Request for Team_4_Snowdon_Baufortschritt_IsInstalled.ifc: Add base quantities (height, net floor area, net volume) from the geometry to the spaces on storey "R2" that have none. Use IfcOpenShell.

First a look at what the model holds.

```python
import ifcopenshell
import ifcopenshell.util.element
import ifcopenshell.util.unit

model = ifcopenshell.open("Team_4_Snowdon_Baufortschritt_IsInstalled.ifc")
print(model.schema)
for unit_type in ("LENGTHUNIT", "AREAUNIT", "VOLUMEUNIT"):
    print(unit_type, ifcopenshell.util.unit.calculate_unit_scale(model, unit_type))
storey = next(s for s in model.by_type("IfcBuildingStorey") if s.Name == "R2")
spaces = [e for e in ifcopenshell.util.element.get_decomposition(storey) if e.is_a("IfcSpace")]
for e in sorted(spaces, key=lambda e: e.id()):
    print(e.id(), e.is_a(), e.Name, list(ifcopenshell.util.element.get_psets(e, qtos_only=True)), sep=" | ")
```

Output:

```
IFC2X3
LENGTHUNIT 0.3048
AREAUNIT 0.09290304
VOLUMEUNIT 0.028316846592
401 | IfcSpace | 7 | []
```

```python
import ifcopenshell
import ifcopenshell.api.pset
import ifcopenshell.geom
import ifcopenshell.util.element
import ifcopenshell.util.shape
import ifcopenshell.util.unit

model = ifcopenshell.open("Team_4_Snowdon_Baufortschritt_IsInstalled.ifc")
unit_scale = ifcopenshell.util.unit.calculate_unit_scale(model)
area_scale = ifcopenshell.util.unit.calculate_unit_scale(model, "AREAUNIT")
volume_scale = ifcopenshell.util.unit.calculate_unit_scale(model, "VOLUMEUNIT")
settings = ifcopenshell.geom.settings()

storey = next(s for s in model.by_type("IfcBuildingStorey") if s.Name == "R2")
spaces = [e for e in ifcopenshell.util.element.get_decomposition(storey) if e.is_a("IfcSpace")]

for e in sorted(spaces, key=lambda e: e.id()):
    if ifcopenshell.util.element.get_psets(e, qtos_only=True, should_inherit=False):
        continue
    # Geometry comes back in metres, in the element's own axes.
    shape = ifcopenshell.geom.create_shape(settings, e)
    values = {
        "Height": ifcopenshell.util.shape.get_z(shape.geometry) / unit_scale,
        "NetFloorArea": ifcopenshell.util.shape.get_footprint_area(shape.geometry) / area_scale,
        "NetVolume": ifcopenshell.util.shape.get_volume(shape.geometry) / volume_scale,
    }
    qto = ifcopenshell.api.pset.add_qto(model, product=e, name="BaseQuantities")
    ifcopenshell.api.pset.edit_qto(model, qto=qto, properties=values)
    print(e.id(), {k: round(v, 3) for k, v in values.items()})

model.write("Team_4_Snowdon_Baufortschritt_IsInstalled_v2.ifc")
```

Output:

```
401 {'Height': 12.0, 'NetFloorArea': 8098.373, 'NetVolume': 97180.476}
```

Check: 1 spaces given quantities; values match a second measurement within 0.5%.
